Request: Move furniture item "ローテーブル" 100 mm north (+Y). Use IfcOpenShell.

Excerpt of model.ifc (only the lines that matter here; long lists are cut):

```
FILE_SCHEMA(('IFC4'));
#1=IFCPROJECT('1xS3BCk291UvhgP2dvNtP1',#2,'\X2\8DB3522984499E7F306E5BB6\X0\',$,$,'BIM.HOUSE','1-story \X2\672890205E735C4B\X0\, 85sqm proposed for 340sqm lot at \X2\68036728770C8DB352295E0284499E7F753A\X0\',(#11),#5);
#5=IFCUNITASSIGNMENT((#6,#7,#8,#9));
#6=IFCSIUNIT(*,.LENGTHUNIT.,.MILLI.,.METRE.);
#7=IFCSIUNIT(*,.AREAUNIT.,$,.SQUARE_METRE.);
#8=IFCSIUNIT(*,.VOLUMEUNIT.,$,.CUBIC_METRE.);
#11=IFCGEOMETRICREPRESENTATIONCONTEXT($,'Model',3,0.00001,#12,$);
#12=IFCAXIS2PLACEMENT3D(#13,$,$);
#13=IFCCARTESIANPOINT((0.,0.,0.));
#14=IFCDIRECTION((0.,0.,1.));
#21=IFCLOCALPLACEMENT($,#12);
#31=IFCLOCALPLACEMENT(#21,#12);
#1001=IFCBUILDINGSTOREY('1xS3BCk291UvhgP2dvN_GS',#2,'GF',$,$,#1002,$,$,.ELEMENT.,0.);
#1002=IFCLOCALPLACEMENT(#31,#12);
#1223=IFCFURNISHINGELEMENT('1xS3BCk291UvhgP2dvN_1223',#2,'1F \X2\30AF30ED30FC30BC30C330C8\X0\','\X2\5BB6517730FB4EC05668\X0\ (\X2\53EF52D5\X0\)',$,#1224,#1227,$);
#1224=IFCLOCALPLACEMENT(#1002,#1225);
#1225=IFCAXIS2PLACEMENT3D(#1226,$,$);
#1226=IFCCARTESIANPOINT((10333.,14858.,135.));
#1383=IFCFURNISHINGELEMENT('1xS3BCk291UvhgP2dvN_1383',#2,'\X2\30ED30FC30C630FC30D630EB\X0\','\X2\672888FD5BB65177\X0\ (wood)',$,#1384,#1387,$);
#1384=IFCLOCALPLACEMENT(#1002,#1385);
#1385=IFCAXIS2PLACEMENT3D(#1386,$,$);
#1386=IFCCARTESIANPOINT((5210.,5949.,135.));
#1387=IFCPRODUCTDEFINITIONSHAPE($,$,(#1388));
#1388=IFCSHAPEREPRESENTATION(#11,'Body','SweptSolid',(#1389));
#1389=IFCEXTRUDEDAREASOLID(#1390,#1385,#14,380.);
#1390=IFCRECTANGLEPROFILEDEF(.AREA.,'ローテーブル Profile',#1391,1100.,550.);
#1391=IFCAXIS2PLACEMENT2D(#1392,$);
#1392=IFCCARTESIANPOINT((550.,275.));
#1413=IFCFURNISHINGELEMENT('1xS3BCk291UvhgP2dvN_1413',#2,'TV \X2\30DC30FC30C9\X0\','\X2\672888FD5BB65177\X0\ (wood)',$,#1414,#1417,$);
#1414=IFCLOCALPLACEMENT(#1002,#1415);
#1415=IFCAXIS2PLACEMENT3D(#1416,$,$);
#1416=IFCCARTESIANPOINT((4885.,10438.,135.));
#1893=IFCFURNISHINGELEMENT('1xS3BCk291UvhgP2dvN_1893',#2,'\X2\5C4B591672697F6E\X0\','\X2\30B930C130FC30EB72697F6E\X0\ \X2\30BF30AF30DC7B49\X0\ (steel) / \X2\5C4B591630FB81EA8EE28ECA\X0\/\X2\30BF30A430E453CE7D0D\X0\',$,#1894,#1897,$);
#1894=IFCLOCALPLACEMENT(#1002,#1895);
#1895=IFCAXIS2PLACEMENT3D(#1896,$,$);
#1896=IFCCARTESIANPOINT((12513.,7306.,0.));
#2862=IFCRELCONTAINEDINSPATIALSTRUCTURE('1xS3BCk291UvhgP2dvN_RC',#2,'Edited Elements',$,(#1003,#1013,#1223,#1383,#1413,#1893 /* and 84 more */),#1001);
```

```python
import ifcopenshell
import ifcopenshell.api.geometry
import ifcopenshell.util.placement
import ifcopenshell.util.unit

model = ifcopenshell.open("model.ifc")
unit_scale = ifcopenshell.util.unit.calculate_unit_scale(model)

item = model.by_id(1383)
matrix = ifcopenshell.util.placement.get_local_placement(item.ObjectPlacement)
matrix[1, 3] += 0.1 / unit_scale
ifcopenshell.api.geometry.edit_object_placement(model, product=item, matrix=matrix, is_si=False)

print(ifcopenshell.util.placement.get_local_placement(item.ObjectPlacement).round(3) + 0.0)

model.write("model_v2.ifc")
```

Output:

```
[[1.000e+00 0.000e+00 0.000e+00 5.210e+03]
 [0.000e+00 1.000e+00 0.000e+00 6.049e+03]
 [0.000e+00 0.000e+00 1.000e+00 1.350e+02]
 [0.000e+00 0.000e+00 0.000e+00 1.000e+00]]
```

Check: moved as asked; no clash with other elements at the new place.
